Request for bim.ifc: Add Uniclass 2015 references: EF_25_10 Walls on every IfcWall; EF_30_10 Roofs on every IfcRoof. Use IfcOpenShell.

First a look at what the model holds.

```python
import ifcopenshell

model = ifcopenshell.open("bim.ifc")
print(model.schema)
print("classifications:", [c.Name for c in model.by_type("IfcClassification")])
for ifc_class in ("IfcDoor", "IfcRoof", "IfcStair", "IfcWall", "IfcWindow"):
    print(ifc_class, len(model.by_type(ifc_class)))
```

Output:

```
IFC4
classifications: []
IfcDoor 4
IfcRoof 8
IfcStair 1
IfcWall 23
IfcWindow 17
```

```python
import ifcopenshell
import ifcopenshell.api.classification

model = ifcopenshell.open("bim.ifc")

system = ifcopenshell.api.classification.add_classification(model, classification="Uniclass 2015")

codes = {
    "IfcWall": ("EF_25_10", "Walls"),
    "IfcRoof": ("EF_30_10", "Roofs"),
}
for ifc_class, (code, name) in codes.items():
    products = model.by_type(ifc_class)
    ifcopenshell.api.classification.add_reference(
        model, products=products, classification=system, identification=code, name=name
    )
    print(code, len(products))

model.write("bim_v2.ifc")
```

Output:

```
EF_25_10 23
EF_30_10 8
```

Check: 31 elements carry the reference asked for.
